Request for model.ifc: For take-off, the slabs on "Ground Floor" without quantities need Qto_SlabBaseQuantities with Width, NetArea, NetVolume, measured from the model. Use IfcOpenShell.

First a look at what the model holds.

```python
import ifcopenshell
import ifcopenshell.util.element
import ifcopenshell.util.unit

model = ifcopenshell.open("model.ifc")
print(model.schema)
for unit_type in ("LENGTHUNIT", "AREAUNIT", "VOLUMEUNIT"):
    print(unit_type, ifcopenshell.util.unit.calculate_unit_scale(model, unit_type))
storey = next(s for s in model.by_type("IfcBuildingStorey") if s.Name == "Ground Floor")
slabs = [e for e in ifcopenshell.util.element.get_decomposition(storey) if e.is_a("IfcSlab")]
for e in sorted(slabs, key=lambda e: e.id()):
    print(e.id(), e.is_a(), e.Name, list(ifcopenshell.util.element.get_psets(e, qtos_only=True)), sep=" | ")
```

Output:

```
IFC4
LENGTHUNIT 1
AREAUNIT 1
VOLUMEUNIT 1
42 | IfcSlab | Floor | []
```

```python
import ifcopenshell
import ifcopenshell.api.pset
import ifcopenshell.geom
import ifcopenshell.util.element
import ifcopenshell.util.shape
import ifcopenshell.util.unit

model = ifcopenshell.open("model.ifc")
unit_scale = ifcopenshell.util.unit.calculate_unit_scale(model)
area_scale = ifcopenshell.util.unit.calculate_unit_scale(model, "AREAUNIT")
volume_scale = ifcopenshell.util.unit.calculate_unit_scale(model, "VOLUMEUNIT")
settings = ifcopenshell.geom.settings()

storey = next(s for s in model.by_type("IfcBuildingStorey") if s.Name == "Ground Floor")
slabs = [e for e in ifcopenshell.util.element.get_decomposition(storey) if e.is_a("IfcSlab")]

for e in sorted(slabs, key=lambda e: e.id()):
    if ifcopenshell.util.element.get_psets(e, qtos_only=True, should_inherit=False):
        continue
    # Geometry comes back in metres, in the element's own axes.
    shape = ifcopenshell.geom.create_shape(settings, e)
    values = {
        "Width": ifcopenshell.util.shape.get_z(shape.geometry) / unit_scale,
        "NetArea": ifcopenshell.util.shape.get_footprint_area(shape.geometry) / area_scale,
        "NetVolume": ifcopenshell.util.shape.get_volume(shape.geometry) / volume_scale,
    }
    qto = ifcopenshell.api.pset.add_qto(model, product=e, name="Qto_SlabBaseQuantities")
    ifcopenshell.api.pset.edit_qto(model, qto=qto, properties=values)
    print(e.id(), {k: round(v, 3) for k, v in values.items()})

model.write("model_updated.ifc")
```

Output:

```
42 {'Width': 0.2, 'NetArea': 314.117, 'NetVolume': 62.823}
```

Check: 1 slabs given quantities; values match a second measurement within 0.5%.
